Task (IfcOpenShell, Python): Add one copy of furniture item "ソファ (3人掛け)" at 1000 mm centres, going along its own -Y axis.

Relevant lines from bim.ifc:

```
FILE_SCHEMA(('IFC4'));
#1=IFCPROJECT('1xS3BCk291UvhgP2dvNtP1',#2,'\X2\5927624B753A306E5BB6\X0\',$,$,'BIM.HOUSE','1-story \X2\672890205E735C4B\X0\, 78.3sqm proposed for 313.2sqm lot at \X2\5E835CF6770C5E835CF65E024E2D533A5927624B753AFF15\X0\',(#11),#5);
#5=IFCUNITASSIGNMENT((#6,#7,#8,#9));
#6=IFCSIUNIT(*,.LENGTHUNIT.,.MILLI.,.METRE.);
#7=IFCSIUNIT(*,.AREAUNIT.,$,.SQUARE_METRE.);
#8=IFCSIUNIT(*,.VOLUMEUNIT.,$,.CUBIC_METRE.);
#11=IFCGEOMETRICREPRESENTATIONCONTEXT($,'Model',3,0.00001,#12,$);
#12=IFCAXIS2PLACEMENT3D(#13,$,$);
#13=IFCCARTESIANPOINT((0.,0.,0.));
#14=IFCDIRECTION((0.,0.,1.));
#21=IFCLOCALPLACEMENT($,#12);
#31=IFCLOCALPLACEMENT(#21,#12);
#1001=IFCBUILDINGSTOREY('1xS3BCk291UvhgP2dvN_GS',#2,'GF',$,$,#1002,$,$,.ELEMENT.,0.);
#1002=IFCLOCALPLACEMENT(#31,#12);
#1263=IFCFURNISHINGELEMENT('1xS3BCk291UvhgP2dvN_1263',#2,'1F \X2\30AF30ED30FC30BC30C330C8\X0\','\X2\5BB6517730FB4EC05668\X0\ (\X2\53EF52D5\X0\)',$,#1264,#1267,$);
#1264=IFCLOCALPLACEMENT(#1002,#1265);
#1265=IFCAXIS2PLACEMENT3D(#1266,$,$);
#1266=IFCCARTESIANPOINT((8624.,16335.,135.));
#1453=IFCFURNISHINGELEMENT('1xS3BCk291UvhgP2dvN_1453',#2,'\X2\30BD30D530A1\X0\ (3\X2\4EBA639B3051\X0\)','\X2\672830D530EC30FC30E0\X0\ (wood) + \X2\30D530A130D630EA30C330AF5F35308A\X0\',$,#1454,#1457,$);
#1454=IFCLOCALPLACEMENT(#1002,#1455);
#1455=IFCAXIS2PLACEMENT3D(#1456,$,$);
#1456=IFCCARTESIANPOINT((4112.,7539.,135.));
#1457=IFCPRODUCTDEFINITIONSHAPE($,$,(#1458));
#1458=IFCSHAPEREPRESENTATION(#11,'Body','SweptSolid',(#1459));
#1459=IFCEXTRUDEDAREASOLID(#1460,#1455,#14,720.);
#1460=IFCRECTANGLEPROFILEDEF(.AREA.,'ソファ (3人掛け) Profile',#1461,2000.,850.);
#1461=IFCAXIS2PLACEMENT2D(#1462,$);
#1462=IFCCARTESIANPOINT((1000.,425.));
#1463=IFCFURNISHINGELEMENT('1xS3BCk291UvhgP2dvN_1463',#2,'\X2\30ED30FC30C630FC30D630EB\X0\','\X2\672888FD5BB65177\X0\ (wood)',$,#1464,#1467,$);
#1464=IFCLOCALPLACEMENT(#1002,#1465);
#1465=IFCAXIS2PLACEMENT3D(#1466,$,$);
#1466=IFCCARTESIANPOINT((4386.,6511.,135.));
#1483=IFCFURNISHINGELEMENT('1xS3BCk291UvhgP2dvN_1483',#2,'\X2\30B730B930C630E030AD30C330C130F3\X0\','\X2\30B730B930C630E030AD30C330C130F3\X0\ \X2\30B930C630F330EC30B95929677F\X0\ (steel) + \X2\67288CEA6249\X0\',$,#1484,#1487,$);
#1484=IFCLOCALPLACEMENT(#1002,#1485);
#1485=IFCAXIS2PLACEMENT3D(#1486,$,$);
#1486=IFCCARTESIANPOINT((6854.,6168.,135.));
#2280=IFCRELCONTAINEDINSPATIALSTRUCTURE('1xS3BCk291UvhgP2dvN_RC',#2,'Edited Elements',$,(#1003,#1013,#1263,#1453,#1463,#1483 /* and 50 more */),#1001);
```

```python
import ifcopenshell
import ifcopenshell.api.geometry
import ifcopenshell.api.root
import ifcopenshell.util.element
import ifcopenshell.util.placement
import ifcopenshell.util.unit

model = ifcopenshell.open("bim.ifc")
unit_scale = ifcopenshell.util.unit.calculate_unit_scale(model)


def reuse_history(source, copy):
    """copy_class also copies each property set's owner history, people and application; keep the originals."""
    for rel in copy.IsDefinedBy:
        if rel.is_a("IfcRelDefinesByProperties") and (history := rel.RelatingPropertyDefinition.OwnerHistory):
            rel.RelatingPropertyDefinition.OwnerHistory = source.OwnerHistory
            ifcopenshell.util.element.remove_deep2(model, history)


source = model.by_guid("1xS3BCk291UvhgP2dvN_1453")
base = ifcopenshell.util.placement.get_local_placement(source.ObjectPlacement)
step = -base[:3, 1] * 1 / unit_scale

for i in range(1, 2):
    copy = ifcopenshell.api.root.copy_class(model, product=source)
    copy.Representation = ifcopenshell.util.element.copy_deep(
        model, source.Representation, exclude=["IfcGeometricRepresentationContext", "IfcRepresentationMap"]
    )
    reuse_history(source, copy)
    matrix = base.copy()
    matrix[:3, 3] += i * step
    print("added at", matrix[:3, 3].round(3) + 0.0)
    ifcopenshell.api.geometry.edit_object_placement(model, product=copy, matrix=matrix, is_si=False)

model.write("bim_updated.ifc")
```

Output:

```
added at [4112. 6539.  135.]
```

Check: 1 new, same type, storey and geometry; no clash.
